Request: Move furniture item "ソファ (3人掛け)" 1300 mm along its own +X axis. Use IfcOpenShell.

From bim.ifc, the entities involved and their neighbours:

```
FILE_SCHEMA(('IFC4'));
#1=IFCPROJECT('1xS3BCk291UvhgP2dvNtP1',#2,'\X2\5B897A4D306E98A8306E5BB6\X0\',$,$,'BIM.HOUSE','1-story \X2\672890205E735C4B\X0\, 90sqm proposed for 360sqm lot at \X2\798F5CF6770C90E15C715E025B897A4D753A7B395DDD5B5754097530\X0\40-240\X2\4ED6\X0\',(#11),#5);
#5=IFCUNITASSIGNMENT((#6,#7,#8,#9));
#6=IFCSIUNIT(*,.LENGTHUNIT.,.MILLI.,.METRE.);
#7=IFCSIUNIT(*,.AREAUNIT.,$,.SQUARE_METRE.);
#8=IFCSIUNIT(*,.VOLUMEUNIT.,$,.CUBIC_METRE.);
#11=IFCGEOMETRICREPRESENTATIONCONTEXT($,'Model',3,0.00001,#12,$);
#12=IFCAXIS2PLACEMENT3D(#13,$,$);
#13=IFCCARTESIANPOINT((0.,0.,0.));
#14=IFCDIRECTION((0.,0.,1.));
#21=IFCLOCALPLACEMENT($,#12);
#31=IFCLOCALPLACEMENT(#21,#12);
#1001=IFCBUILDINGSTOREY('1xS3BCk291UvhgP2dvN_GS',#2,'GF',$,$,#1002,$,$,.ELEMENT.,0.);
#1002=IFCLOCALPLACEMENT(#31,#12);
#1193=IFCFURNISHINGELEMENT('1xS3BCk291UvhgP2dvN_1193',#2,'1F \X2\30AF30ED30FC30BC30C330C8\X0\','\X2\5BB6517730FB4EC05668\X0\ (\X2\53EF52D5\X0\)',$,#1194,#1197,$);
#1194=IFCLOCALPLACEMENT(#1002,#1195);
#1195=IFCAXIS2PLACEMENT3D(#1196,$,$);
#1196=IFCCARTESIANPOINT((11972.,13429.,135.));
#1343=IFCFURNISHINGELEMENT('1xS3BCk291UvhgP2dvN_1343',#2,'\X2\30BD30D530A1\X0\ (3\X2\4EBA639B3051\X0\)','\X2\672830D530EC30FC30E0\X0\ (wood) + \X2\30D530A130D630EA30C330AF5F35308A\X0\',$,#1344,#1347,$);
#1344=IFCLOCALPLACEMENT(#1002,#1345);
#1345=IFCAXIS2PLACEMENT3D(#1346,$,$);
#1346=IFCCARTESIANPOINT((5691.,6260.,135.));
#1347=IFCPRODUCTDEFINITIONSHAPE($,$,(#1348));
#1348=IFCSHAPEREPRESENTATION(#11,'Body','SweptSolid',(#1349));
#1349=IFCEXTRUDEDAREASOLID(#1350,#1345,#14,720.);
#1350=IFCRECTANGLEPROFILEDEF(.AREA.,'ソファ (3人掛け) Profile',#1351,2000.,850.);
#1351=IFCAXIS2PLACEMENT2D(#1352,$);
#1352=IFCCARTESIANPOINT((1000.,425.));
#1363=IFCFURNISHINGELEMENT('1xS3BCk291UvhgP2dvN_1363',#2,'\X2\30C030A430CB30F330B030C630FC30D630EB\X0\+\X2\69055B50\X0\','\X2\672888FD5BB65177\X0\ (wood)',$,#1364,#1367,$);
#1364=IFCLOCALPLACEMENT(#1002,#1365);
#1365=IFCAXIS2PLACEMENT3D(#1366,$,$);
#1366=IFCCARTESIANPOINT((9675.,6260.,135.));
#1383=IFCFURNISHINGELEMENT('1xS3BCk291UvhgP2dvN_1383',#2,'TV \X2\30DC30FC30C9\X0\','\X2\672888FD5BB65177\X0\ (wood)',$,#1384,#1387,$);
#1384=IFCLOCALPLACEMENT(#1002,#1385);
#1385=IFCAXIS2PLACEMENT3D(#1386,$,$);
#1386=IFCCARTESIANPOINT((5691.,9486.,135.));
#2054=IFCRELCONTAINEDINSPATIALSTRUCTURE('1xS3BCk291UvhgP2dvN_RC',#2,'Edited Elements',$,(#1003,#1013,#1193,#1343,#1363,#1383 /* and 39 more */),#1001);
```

```python
import ifcopenshell
import ifcopenshell.api.geometry
import ifcopenshell.util.placement
import ifcopenshell.util.unit

model = ifcopenshell.open("bim.ifc")
unit_scale = ifcopenshell.util.unit.calculate_unit_scale(model)

item = model.by_id(1343)
matrix = ifcopenshell.util.placement.get_local_placement(item.ObjectPlacement)
matrix[:3, 3] += matrix[:3, 0] * 1.3 / unit_scale
ifcopenshell.api.geometry.edit_object_placement(model, product=item, matrix=matrix, is_si=False)

print(ifcopenshell.util.placement.get_local_placement(item.ObjectPlacement).round(3) + 0.0)

model.write("bim_rev.ifc")
```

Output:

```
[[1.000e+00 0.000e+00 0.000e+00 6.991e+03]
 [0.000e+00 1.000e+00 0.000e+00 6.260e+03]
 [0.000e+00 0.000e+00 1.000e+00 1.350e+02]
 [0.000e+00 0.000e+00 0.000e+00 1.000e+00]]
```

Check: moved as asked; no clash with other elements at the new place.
